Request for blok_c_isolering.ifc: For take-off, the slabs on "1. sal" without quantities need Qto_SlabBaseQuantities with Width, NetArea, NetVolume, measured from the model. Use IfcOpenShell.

First a look at what the model holds.

```python
import ifcopenshell
import ifcopenshell.util.element
import ifcopenshell.util.unit

model = ifcopenshell.open("blok_c_isolering.ifc")
print(model.schema)
for unit_type in ("LENGTHUNIT", "AREAUNIT", "VOLUMEUNIT"):
    print(unit_type, ifcopenshell.util.unit.calculate_unit_scale(model, unit_type))
storey = next(s for s in model.by_type("IfcBuildingStorey") if s.Name == "1. sal")
slabs = [e for e in ifcopenshell.util.element.get_decomposition(storey) if e.is_a("IfcSlab")]
for e in sorted(slabs, key=lambda e: e.id()):
    print(e.id(), e.is_a(), e.Name, list(ifcopenshell.util.element.get_psets(e, qtos_only=True)), sep=" | ")
```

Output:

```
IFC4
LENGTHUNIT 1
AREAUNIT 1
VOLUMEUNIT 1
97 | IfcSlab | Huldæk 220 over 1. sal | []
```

```python
import ifcopenshell
import ifcopenshell.api.pset
import ifcopenshell.geom
import ifcopenshell.util.element
import ifcopenshell.util.shape
import ifcopenshell.util.unit

model = ifcopenshell.open("blok_c_isolering.ifc")
unit_scale = ifcopenshell.util.unit.calculate_unit_scale(model)
area_scale = ifcopenshell.util.unit.calculate_unit_scale(model, "AREAUNIT")
volume_scale = ifcopenshell.util.unit.calculate_unit_scale(model, "VOLUMEUNIT")
settings = ifcopenshell.geom.settings()

storey = next(s for s in model.by_type("IfcBuildingStorey") if s.Name == "1. sal")
slabs = [e for e in ifcopenshell.util.element.get_decomposition(storey) if e.is_a("IfcSlab")]

for e in sorted(slabs, key=lambda e: e.id()):
    if ifcopenshell.util.element.get_psets(e, qtos_only=True, should_inherit=False):
        continue
    # Geometry comes back in metres, in the element's own axes.
    shape = ifcopenshell.geom.create_shape(settings, e)
    values = {
        "Width": ifcopenshell.util.shape.get_z(shape.geometry) / unit_scale,
        "NetArea": ifcopenshell.util.shape.get_footprint_area(shape.geometry) / area_scale,
        "NetVolume": ifcopenshell.util.shape.get_volume(shape.geometry) / volume_scale,
    }
    qto = ifcopenshell.api.pset.add_qto(model, product=e, name="Qto_SlabBaseQuantities")
    ifcopenshell.api.pset.edit_qto(model, qto=qto, properties=values)
    print(e.id(), {k: round(v, 3) for k, v in values.items()})

model.write("blok_c_isolering_v2.ifc")
```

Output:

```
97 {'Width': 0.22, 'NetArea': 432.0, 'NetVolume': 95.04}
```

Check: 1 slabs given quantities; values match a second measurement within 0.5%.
